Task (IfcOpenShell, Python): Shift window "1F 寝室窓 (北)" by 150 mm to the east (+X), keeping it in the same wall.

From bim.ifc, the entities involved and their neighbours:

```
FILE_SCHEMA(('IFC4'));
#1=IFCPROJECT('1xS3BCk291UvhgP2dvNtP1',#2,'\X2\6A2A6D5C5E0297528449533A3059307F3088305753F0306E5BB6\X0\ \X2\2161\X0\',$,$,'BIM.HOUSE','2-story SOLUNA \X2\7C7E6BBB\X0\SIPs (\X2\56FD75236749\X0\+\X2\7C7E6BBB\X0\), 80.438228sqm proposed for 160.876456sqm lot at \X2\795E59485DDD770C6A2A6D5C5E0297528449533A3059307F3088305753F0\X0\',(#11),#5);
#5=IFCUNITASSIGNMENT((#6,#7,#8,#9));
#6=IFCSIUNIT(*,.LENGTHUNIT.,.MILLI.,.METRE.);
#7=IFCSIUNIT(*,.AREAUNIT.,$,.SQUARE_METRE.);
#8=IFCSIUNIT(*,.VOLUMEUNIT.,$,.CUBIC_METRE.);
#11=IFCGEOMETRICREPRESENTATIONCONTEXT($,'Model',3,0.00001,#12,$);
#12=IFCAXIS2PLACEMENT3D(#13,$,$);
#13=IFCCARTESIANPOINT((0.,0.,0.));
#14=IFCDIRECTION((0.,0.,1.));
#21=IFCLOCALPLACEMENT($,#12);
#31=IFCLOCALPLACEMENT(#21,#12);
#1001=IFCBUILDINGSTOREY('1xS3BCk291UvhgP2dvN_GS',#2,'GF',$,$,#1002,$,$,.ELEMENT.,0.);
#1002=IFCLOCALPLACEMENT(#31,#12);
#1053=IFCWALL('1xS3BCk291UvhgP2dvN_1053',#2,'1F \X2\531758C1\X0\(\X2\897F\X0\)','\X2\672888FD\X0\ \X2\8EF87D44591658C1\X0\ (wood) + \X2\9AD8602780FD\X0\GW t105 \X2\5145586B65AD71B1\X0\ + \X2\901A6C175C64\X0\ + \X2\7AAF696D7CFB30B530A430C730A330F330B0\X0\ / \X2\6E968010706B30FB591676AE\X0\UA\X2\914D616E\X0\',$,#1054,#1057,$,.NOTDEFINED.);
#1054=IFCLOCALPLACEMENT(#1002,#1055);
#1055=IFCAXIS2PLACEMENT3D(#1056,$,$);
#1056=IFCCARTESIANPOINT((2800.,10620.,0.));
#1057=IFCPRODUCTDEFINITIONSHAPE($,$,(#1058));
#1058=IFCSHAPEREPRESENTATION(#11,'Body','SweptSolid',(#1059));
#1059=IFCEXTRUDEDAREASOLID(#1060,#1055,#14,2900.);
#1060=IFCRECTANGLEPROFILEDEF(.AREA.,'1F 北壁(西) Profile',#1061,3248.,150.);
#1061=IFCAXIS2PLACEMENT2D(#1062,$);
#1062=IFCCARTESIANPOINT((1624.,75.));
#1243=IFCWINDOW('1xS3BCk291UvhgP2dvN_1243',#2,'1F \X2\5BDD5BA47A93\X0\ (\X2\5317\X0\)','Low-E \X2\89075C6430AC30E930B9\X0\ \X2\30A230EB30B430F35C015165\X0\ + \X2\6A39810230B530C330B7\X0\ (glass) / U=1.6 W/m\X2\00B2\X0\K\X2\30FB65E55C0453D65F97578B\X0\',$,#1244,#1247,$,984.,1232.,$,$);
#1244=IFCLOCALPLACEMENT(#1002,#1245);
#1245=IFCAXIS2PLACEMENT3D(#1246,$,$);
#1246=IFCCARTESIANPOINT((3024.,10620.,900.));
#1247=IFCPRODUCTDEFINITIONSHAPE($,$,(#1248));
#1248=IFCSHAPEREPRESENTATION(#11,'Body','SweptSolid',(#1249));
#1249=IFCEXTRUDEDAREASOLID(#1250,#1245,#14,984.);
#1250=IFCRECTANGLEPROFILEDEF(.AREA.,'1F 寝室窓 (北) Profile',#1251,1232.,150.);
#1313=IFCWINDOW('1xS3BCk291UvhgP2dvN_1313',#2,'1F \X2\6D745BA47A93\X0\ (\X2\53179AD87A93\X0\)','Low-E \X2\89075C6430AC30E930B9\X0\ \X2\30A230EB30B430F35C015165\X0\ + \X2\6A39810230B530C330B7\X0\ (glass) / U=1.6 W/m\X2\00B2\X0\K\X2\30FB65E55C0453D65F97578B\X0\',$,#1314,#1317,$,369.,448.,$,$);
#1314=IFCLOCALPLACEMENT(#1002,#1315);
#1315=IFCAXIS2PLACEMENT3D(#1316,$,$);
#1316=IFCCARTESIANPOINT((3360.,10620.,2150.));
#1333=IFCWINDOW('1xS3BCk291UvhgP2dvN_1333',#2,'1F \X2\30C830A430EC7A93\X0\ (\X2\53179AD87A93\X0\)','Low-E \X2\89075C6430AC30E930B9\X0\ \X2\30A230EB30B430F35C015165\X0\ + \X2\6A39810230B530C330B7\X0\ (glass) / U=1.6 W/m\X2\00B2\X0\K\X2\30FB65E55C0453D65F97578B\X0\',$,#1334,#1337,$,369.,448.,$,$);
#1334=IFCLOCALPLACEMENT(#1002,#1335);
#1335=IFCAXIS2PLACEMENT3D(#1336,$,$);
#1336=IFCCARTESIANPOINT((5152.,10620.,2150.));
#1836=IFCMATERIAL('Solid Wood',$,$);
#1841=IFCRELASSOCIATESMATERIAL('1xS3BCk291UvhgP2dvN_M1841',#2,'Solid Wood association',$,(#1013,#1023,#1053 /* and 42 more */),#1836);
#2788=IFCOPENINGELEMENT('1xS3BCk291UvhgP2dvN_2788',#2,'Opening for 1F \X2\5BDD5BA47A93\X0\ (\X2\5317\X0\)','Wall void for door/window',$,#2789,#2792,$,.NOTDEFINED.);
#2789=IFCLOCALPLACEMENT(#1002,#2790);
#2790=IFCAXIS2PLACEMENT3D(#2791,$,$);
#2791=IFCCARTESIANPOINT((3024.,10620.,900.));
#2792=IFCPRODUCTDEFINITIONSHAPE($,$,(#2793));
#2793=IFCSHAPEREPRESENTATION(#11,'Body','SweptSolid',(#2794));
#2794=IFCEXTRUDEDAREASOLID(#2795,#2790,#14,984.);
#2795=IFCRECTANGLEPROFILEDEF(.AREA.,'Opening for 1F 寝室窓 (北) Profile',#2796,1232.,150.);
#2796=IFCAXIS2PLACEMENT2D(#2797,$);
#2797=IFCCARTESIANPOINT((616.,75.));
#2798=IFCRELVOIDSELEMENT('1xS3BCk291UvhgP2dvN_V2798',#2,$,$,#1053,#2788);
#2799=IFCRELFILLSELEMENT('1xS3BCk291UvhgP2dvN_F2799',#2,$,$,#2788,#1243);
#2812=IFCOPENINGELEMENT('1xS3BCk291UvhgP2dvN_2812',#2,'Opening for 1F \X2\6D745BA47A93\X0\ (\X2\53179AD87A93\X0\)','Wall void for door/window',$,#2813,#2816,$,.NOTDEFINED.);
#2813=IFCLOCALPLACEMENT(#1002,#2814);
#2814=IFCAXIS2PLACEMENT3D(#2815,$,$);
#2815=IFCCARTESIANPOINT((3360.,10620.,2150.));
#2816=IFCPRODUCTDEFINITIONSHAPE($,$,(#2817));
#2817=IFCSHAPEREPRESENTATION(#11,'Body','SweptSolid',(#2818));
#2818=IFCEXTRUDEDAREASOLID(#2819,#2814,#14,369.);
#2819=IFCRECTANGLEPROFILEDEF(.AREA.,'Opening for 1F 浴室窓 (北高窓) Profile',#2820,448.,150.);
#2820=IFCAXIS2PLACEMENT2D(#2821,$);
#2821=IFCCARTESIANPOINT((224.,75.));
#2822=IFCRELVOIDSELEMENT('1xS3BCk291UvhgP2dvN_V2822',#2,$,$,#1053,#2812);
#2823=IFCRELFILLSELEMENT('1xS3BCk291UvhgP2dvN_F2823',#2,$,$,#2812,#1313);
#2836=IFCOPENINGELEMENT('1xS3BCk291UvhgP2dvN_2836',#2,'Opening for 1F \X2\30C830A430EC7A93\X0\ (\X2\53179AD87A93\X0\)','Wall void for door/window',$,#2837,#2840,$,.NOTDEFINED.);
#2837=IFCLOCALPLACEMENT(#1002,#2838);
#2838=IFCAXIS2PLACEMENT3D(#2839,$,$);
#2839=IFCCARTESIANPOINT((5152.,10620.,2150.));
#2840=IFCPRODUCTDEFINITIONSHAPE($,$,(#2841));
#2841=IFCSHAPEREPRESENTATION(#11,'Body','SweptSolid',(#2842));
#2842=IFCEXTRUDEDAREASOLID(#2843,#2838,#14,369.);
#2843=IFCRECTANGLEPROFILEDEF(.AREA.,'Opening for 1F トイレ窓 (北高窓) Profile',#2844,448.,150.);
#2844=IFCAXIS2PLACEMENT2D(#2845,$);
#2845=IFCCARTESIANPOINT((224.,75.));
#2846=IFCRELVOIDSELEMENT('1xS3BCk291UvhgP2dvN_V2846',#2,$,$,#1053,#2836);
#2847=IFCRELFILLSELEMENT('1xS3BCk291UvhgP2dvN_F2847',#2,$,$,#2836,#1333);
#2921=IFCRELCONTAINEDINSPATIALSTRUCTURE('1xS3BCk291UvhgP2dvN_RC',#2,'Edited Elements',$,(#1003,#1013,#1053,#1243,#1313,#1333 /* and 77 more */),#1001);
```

```python
import ifcopenshell
import ifcopenshell.api.geometry
import ifcopenshell.util.placement
import ifcopenshell.util.unit

model = ifcopenshell.open("bim.ifc")
unit_scale = ifcopenshell.util.unit.calculate_unit_scale(model)

window = model.by_id(1243)
opening = window.FillsVoids[0].RelatingOpeningElement
wall = opening.VoidsElements[0].RelatingBuildingElement

wall_matrix = ifcopenshell.util.placement.get_local_placement(wall.ObjectPlacement)
shift = wall_matrix[:3, 0] * 0.15 / unit_scale
before = ifcopenshell.util.placement.get_local_placement(window.ObjectPlacement)[:3, 3].copy()

# The window is not placed relative to its opening, so move both.
for product in (opening, window):
    matrix = ifcopenshell.util.placement.get_local_placement(product.ObjectPlacement)
    matrix[:3, 3] += shift
    ifcopenshell.api.geometry.edit_object_placement(model, product=product, matrix=matrix, is_si=False)

after = ifcopenshell.util.placement.get_local_placement(window.ObjectPlacement)[:3, 3]
print("window moved by", (after - before).round(3) + 0.0)

model.write("bim_v2.ifc")
```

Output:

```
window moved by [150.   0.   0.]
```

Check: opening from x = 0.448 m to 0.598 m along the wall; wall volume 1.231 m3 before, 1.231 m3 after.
